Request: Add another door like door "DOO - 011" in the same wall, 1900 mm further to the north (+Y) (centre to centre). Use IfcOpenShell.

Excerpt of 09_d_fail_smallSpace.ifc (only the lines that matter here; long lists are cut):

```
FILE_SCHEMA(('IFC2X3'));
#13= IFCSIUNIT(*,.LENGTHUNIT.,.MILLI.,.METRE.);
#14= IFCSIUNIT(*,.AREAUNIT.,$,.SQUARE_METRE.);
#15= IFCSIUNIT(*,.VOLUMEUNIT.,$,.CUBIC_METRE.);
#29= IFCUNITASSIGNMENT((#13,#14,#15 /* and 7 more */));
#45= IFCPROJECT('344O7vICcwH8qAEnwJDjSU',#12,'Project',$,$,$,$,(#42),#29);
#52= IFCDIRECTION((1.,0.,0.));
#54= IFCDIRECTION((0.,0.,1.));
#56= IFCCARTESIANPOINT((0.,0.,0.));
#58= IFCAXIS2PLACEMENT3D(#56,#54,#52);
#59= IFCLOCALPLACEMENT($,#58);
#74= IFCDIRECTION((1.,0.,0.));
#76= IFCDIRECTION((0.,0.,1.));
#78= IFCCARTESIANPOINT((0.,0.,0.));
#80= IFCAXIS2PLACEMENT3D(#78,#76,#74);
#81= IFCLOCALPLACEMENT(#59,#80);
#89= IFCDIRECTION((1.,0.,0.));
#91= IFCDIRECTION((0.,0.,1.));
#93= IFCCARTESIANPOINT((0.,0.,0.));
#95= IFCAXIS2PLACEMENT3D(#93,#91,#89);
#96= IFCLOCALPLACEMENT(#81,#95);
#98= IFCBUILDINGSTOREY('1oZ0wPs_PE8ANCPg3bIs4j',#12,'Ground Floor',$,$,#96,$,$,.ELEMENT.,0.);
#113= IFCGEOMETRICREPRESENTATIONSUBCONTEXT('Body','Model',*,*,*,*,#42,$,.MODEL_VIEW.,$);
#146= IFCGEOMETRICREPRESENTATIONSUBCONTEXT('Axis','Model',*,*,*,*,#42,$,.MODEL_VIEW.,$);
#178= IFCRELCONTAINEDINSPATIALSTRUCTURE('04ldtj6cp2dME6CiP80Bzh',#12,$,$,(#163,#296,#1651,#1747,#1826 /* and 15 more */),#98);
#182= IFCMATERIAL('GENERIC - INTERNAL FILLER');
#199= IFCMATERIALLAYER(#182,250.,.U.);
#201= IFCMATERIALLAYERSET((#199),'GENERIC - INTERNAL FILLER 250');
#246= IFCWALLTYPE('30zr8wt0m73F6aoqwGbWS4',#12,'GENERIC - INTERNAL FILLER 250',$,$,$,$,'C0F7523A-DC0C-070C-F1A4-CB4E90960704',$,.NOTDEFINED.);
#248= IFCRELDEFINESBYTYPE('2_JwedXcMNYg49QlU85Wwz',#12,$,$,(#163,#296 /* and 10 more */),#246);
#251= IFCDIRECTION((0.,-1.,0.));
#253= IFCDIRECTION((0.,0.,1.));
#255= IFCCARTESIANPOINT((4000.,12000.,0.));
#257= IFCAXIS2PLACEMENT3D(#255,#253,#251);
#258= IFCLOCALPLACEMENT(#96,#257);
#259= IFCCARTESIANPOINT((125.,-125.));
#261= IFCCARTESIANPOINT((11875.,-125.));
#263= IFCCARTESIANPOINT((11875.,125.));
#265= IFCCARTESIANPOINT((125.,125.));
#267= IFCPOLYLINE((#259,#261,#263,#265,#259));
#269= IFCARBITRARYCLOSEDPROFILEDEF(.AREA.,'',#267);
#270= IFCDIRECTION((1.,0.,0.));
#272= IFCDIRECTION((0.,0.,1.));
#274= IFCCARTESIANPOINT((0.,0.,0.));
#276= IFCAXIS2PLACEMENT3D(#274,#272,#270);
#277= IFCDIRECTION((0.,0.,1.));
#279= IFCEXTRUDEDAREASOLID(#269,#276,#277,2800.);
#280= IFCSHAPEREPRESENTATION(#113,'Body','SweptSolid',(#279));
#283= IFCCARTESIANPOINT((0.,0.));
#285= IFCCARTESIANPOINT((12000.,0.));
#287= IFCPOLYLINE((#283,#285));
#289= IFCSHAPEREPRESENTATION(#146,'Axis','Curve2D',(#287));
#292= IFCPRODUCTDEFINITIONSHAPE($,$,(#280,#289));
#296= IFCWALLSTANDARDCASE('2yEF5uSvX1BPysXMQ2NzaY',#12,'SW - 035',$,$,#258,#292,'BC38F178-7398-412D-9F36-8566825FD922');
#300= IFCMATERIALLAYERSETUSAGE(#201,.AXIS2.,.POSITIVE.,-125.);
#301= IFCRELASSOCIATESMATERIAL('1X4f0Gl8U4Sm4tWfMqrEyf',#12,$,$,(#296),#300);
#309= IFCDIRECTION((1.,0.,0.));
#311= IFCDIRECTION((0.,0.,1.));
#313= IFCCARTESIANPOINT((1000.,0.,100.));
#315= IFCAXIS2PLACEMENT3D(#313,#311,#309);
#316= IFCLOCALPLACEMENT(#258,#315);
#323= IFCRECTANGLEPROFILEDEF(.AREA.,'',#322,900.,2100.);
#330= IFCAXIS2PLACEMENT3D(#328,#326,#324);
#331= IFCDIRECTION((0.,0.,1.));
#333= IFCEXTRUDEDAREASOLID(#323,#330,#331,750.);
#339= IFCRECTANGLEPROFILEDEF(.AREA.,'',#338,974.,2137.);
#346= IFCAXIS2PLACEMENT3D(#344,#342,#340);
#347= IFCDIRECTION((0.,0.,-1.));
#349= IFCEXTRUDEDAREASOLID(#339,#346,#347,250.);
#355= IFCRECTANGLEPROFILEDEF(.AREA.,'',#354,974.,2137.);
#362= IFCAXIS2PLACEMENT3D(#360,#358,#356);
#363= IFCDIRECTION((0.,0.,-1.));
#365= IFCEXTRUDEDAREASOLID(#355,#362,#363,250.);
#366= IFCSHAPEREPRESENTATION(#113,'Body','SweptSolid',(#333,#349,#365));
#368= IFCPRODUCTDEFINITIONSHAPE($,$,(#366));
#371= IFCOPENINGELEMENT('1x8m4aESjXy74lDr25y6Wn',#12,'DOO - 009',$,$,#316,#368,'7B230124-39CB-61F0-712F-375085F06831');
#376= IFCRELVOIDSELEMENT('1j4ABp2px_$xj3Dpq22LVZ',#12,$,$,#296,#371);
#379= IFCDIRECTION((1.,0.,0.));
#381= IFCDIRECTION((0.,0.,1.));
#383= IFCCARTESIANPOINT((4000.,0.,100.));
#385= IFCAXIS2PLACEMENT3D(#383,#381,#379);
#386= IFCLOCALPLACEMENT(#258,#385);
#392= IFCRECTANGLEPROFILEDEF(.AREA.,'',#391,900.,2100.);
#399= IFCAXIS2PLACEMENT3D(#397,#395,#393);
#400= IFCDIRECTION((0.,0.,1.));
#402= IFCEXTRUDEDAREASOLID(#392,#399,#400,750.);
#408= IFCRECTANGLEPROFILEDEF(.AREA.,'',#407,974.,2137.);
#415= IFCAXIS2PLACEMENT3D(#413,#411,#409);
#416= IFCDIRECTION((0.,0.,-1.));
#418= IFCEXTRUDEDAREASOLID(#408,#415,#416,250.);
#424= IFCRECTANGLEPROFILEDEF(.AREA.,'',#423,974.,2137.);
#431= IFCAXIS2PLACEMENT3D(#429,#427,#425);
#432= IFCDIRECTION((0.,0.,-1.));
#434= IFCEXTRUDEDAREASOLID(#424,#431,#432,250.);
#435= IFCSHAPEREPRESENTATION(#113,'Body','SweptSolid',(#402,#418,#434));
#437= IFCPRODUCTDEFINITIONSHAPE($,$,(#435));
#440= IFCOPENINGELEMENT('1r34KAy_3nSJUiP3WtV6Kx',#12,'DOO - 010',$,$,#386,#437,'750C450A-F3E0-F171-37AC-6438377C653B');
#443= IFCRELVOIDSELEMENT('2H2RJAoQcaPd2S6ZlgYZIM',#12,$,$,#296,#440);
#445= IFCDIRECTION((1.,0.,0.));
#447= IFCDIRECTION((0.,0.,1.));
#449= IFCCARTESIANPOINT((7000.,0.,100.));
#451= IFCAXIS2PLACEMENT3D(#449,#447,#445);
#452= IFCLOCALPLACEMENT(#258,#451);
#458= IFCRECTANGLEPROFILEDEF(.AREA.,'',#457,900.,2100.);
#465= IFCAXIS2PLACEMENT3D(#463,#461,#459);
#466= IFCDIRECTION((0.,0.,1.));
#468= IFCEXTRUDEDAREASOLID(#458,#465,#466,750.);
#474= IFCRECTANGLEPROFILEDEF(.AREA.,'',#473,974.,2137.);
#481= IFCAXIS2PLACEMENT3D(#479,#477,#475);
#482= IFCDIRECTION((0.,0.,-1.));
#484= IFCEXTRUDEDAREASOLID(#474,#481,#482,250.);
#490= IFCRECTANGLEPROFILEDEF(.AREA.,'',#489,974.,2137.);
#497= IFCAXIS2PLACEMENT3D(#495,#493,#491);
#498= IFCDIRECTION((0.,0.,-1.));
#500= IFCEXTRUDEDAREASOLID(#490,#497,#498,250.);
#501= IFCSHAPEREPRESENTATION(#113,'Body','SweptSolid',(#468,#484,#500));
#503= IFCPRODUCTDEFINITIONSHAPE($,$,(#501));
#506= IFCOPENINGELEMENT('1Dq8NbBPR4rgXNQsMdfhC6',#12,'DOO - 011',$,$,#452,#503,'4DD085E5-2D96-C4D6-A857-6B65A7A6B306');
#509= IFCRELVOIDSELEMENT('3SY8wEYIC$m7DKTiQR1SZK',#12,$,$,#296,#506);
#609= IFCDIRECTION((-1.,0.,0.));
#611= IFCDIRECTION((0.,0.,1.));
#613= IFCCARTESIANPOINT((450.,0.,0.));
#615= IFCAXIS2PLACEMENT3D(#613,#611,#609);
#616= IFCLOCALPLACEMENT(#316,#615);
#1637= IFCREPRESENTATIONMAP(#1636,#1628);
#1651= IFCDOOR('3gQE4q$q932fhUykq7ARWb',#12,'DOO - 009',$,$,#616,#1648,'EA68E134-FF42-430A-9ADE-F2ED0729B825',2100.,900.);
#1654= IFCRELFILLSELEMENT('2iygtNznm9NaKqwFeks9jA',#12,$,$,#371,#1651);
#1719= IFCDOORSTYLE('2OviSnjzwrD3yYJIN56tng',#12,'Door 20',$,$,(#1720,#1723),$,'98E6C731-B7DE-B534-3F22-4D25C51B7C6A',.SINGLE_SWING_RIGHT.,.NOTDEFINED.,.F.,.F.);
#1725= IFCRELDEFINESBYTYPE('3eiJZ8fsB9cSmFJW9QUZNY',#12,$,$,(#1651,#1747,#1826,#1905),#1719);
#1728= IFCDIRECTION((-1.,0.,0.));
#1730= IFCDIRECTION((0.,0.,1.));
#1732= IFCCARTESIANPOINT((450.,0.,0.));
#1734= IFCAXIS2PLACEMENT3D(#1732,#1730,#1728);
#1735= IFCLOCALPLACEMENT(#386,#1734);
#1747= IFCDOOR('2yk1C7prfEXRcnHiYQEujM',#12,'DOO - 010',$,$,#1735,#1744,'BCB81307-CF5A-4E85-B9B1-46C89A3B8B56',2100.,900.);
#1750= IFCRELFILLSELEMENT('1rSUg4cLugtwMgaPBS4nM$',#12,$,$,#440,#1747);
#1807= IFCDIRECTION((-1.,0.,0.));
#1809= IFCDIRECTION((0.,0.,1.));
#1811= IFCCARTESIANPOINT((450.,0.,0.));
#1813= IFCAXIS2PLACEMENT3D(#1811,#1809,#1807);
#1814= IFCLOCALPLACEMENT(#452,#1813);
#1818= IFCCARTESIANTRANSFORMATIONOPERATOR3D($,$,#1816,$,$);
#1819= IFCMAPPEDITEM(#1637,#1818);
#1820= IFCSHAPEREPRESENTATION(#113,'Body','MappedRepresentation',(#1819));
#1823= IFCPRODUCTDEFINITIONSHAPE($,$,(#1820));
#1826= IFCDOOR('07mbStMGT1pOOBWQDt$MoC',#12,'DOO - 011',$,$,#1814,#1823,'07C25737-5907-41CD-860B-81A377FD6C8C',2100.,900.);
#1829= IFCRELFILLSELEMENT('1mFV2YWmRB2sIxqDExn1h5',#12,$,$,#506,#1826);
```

```python
import ifcopenshell
import ifcopenshell.api.feature
import ifcopenshell.api.geometry
import ifcopenshell.api.root
import ifcopenshell.geom
import ifcopenshell.util.element
import ifcopenshell.util.placement
import ifcopenshell.util.shape

model = ifcopenshell.open("09_d_fail_smallSpace.ifc")
settings = ifcopenshell.geom.settings()


def volume(element):
    """Net volume in cubic metres, openings subtracted."""
    shape = ifcopenshell.geom.create_shape(settings, element)
    return ifcopenshell.util.shape.get_volume(shape.geometry)


def reuse_history(source, copy):
    """copy_class also copies each property set's owner history, people and application; keep the originals."""
    for rel in copy.IsDefinedBy:
        if rel.is_a("IfcRelDefinesByProperties") and (history := rel.RelatingPropertyDefinition.OwnerHistory):
            rel.RelatingPropertyDefinition.OwnerHistory = source.OwnerHistory
            ifcopenshell.util.element.remove_deep2(model, history)


door = model.by_guid("07mbStMGT1pOOBWQDt$MoC")
opening = door.FillsVoids[0].RelatingOpeningElement
wall = opening.VoidsElements[0].RelatingBuildingElement
before = volume(wall)
shift = ifcopenshell.util.placement.get_local_placement(wall.ObjectPlacement)[:3, 0] * -1900.0

# copy_class copies the void relationship, type, container and properties, but no geometry.
new_opening = ifcopenshell.api.root.copy_class(model, product=opening)
new_opening.Representation = ifcopenshell.util.element.copy_deep(
    model, opening.Representation, exclude=["IfcGeometricRepresentationContext", "IfcRepresentationMap"]
)
new_opening.Tag = None
new_door = ifcopenshell.api.root.copy_class(model, product=door)
new_door.Representation = ifcopenshell.util.element.copy_deep(
    model, door.Representation, exclude=["IfcGeometricRepresentationContext", "IfcRepresentationMap"]
)
new_door.Tag = None
reuse_history(door, new_door)
fills = ifcopenshell.api.feature.add_filling(model, opening=new_opening, element=new_door)
fills.OwnerHistory = new_door.OwnerHistory  # required in IFC2X3

for old, new in ((opening, new_opening), (door, new_door)):
    matrix = ifcopenshell.util.placement.get_local_placement(old.ObjectPlacement)
    matrix[:3, 3] += shift
    ifcopenshell.api.geometry.edit_object_placement(model, product=new, matrix=matrix, is_si=False)

after = volume(wall)

print(f"wall volume {before:.3f} -> {after:.3f} m3")

model.write("09_d_fail_smallSpace_edited.ifc")
```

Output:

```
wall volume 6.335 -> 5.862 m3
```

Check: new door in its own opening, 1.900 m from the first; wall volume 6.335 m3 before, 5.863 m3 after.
